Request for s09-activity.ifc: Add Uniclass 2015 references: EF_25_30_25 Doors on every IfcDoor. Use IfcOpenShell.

First a look at what the model holds.

```python
import ifcopenshell

model = ifcopenshell.open("s09-activity.ifc")
print(model.schema)
print("classifications:", [c.Name for c in model.by_type("IfcClassification")])
for ifc_class in ("IfcDoor", "IfcRoof", "IfcStair", "IfcWall", "IfcWindow"):
    print(ifc_class, len(model.by_type(ifc_class)))
```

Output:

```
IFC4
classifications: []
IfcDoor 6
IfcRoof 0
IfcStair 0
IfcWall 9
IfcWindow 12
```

```python
import ifcopenshell
import ifcopenshell.api.classification

model = ifcopenshell.open("s09-activity.ifc")

system = ifcopenshell.api.classification.add_classification(model, classification="Uniclass 2015")

codes = {
    "IfcDoor": ("EF_25_30_25", "Doors"),
}
for ifc_class, (code, name) in codes.items():
    products = model.by_type(ifc_class)
    ifcopenshell.api.classification.add_reference(
        model, products=products, classification=system, identification=code, name=name
    )
    print(code, len(products))

model.write("s09-activity_updated.ifc")
```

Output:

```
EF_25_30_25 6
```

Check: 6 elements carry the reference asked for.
